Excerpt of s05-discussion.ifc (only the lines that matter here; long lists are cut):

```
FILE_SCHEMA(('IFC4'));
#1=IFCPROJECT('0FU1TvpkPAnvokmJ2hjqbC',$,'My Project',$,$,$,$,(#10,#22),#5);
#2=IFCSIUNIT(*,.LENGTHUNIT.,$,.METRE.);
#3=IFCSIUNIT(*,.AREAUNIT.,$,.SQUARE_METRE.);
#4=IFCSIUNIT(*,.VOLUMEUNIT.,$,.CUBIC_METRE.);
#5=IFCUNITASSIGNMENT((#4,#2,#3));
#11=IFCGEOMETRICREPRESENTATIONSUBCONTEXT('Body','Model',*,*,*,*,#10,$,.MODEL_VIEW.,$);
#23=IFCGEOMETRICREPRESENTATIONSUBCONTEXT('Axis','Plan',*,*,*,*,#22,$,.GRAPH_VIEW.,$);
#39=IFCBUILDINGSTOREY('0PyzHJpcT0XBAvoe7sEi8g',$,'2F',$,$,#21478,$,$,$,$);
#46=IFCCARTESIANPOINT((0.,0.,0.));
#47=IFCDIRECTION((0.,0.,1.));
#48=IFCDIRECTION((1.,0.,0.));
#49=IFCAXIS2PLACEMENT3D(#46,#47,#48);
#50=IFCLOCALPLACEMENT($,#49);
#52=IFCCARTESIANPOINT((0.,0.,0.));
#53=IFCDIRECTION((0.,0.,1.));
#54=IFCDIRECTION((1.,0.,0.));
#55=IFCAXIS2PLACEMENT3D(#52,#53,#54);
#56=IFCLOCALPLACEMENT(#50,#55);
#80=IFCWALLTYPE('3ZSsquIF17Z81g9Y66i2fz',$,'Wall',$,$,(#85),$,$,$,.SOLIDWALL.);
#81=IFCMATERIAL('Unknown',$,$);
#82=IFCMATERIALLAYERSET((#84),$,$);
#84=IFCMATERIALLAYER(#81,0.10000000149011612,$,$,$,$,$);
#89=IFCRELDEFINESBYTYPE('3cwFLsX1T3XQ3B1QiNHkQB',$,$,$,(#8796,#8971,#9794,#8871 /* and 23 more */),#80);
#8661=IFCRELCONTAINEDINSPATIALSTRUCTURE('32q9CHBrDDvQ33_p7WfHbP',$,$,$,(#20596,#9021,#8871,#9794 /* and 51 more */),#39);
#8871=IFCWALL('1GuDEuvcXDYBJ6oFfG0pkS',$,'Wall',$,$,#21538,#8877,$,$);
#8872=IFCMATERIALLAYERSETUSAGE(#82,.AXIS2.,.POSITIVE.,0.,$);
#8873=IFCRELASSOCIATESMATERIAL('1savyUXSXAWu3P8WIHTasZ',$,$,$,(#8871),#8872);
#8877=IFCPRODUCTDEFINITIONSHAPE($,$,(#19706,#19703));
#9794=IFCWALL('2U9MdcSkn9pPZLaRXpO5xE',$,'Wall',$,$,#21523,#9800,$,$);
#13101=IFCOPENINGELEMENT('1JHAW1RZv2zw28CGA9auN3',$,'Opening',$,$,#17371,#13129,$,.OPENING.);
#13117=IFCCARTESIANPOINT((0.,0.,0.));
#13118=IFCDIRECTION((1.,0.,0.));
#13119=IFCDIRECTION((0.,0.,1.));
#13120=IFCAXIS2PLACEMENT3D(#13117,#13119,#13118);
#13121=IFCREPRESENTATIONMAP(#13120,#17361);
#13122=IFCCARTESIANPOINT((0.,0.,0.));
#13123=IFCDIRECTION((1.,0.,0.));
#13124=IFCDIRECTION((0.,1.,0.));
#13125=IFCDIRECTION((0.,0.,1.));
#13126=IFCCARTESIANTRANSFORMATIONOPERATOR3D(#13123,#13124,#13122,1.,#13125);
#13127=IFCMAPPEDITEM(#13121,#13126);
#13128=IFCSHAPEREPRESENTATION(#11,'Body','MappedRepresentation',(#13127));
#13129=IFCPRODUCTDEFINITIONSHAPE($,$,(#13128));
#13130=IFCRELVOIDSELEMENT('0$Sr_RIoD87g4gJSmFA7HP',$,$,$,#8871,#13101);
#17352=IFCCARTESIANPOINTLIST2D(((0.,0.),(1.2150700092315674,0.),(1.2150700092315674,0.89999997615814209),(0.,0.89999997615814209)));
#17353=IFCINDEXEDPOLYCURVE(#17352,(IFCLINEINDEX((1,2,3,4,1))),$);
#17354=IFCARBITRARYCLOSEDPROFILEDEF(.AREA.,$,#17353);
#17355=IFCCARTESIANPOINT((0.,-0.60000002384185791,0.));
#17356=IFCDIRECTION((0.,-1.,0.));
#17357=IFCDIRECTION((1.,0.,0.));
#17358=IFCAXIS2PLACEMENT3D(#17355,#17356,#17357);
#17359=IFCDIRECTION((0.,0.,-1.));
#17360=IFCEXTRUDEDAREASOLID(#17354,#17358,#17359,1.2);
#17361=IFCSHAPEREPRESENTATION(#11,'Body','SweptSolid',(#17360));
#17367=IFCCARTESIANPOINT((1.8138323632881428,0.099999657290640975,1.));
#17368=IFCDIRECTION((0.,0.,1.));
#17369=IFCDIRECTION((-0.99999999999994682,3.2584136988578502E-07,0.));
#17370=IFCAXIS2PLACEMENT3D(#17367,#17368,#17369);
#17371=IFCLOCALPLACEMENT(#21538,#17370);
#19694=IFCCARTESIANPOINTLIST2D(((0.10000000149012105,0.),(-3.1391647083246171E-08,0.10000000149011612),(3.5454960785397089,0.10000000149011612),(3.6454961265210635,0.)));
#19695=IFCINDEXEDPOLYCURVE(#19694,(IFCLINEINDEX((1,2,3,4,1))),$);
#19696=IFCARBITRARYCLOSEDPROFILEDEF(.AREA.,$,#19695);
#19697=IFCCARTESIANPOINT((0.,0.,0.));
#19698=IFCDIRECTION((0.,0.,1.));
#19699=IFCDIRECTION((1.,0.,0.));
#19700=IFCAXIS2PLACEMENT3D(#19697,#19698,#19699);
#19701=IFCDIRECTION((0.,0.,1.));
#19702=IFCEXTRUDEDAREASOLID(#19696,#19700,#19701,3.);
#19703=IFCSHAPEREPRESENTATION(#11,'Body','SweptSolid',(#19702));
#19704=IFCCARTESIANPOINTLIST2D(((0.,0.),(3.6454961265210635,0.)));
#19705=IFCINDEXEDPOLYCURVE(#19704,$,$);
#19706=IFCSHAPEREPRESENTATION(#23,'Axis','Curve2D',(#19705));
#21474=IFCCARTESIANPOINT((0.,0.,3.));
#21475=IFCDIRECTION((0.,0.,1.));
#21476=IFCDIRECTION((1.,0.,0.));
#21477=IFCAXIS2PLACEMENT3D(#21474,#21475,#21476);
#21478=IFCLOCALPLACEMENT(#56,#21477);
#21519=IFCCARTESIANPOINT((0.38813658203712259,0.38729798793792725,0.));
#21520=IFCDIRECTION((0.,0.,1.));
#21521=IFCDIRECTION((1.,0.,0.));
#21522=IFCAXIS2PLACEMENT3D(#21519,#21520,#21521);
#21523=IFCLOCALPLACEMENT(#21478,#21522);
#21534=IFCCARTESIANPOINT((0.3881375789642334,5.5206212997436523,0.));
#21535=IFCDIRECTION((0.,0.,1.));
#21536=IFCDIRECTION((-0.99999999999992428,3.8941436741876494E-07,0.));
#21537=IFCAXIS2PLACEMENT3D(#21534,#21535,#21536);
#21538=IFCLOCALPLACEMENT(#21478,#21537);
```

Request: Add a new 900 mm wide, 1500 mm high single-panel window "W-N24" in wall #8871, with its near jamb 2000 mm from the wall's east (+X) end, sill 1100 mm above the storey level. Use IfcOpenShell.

```python
import numpy as np
import ifcopenshell
import ifcopenshell.api.feature
import ifcopenshell.api.geometry
import ifcopenshell.api.root
import ifcopenshell.api.spatial
import ifcopenshell.geom
import ifcopenshell.util.element
import ifcopenshell.util.placement
import ifcopenshell.util.representation
import ifcopenshell.util.shape
import ifcopenshell.util.unit

model = ifcopenshell.open("s05-discussion.ifc")
unit_scale = ifcopenshell.util.unit.calculate_unit_scale(model)
settings = ifcopenshell.geom.settings()


def volume(element):
    """Net volume in cubic metres, openings subtracted."""
    shape = ifcopenshell.geom.create_shape(settings, element)
    return ifcopenshell.util.shape.get_volume(shape.geometry)


wall = model.by_guid("1GuDEuvcXDYBJ6oFfG0pkS")
storey = ifcopenshell.util.element.get_container(wall, ifc_class="IfcBuildingStorey")
context = ifcopenshell.util.representation.get_context(model, "Model", "Body", "MODEL_VIEW")
before = volume(wall)

width, height, from_end, sill = 0.9, 1.5, 2, 1.1  # metres

# The wall runs along its own X axis, and the end named is its -X end.
wall_shape = ifcopenshell.geom.create_shape(settings, wall)
x, y, z = ifcopenshell.util.shape.get_vertices(wall_shape.geometry).T
start = x.min() + from_end
face, thickness = float(y.min()), float(y.max() - y.min())
wall_matrix = ifcopenshell.util.placement.get_local_placement(wall.ObjectPlacement)
level = ifcopenshell.util.placement.get_local_placement(storey.ObjectPlacement)[2, 3]


def in_wall(x, y):
    """Placement at x, y metres in the wall's axes, at sill height."""
    matrix = wall_matrix.copy()
    matrix[:, 3] = wall_matrix @ np.array([x / unit_scale, y / unit_scale, 0.0, 1.0])
    matrix[2, 3] = level + sill / unit_scale
    return matrix


# Opening: a box that overshoots both wall faces by 50 mm.
opening = ifcopenshell.api.root.create_entity(model, ifc_class="IfcOpeningElement", predefined_type="OPENING")
box = ifcopenshell.api.geometry.add_wall_representation(
    model, context=context, length=width, height=height, thickness=thickness + 0.1
)
ifcopenshell.api.geometry.assign_representation(model, product=opening, representation=box)
ifcopenshell.api.geometry.edit_object_placement(model, product=opening, matrix=in_wall(start, face - 0.05), is_si=False)
ifcopenshell.api.feature.add_feature(model, feature=opening, element=wall)

window = ifcopenshell.api.root.create_entity(model, ifc_class="IfcWindow", name="W-N24", predefined_type="WINDOW")
window.OverallWidth, window.OverallHeight = width / unit_scale, height / unit_scale
window.PartitioningType = "SINGLE_PANEL"
body = ifcopenshell.api.geometry.add_window_representation(
    model,
    context=context,
    overall_width=window.OverallWidth,
    overall_height=window.OverallHeight,
    partition_type="SINGLE_PANEL",
)
ifcopenshell.api.geometry.assign_representation(model, product=window, representation=body)
ifcopenshell.api.spatial.assign_container(model, products=[window], relating_structure=storey)
ifcopenshell.api.feature.add_filling(model, opening=opening, element=window)

# Centre the window in the wall's thickness.
ifcopenshell.api.geometry.edit_object_placement(model, product=window, matrix=in_wall(start, face), is_si=False)
window_shape = ifcopenshell.geom.create_shape(settings, window)
depth = ifcopenshell.util.shape.get_vertices(window_shape.geometry)[:, 1]
offset = face + thickness / 2 - (depth.min() + depth.max()) / 2
ifcopenshell.api.geometry.edit_object_placement(model, product=window, matrix=in_wall(start, offset), is_si=False)

after = volume(wall)

print(f"wall volume {before:.3f} -> {after:.3f} m3")

model.write("s05-discussion_rev.ifc")
```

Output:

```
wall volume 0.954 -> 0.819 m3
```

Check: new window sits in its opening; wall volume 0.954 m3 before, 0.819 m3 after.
